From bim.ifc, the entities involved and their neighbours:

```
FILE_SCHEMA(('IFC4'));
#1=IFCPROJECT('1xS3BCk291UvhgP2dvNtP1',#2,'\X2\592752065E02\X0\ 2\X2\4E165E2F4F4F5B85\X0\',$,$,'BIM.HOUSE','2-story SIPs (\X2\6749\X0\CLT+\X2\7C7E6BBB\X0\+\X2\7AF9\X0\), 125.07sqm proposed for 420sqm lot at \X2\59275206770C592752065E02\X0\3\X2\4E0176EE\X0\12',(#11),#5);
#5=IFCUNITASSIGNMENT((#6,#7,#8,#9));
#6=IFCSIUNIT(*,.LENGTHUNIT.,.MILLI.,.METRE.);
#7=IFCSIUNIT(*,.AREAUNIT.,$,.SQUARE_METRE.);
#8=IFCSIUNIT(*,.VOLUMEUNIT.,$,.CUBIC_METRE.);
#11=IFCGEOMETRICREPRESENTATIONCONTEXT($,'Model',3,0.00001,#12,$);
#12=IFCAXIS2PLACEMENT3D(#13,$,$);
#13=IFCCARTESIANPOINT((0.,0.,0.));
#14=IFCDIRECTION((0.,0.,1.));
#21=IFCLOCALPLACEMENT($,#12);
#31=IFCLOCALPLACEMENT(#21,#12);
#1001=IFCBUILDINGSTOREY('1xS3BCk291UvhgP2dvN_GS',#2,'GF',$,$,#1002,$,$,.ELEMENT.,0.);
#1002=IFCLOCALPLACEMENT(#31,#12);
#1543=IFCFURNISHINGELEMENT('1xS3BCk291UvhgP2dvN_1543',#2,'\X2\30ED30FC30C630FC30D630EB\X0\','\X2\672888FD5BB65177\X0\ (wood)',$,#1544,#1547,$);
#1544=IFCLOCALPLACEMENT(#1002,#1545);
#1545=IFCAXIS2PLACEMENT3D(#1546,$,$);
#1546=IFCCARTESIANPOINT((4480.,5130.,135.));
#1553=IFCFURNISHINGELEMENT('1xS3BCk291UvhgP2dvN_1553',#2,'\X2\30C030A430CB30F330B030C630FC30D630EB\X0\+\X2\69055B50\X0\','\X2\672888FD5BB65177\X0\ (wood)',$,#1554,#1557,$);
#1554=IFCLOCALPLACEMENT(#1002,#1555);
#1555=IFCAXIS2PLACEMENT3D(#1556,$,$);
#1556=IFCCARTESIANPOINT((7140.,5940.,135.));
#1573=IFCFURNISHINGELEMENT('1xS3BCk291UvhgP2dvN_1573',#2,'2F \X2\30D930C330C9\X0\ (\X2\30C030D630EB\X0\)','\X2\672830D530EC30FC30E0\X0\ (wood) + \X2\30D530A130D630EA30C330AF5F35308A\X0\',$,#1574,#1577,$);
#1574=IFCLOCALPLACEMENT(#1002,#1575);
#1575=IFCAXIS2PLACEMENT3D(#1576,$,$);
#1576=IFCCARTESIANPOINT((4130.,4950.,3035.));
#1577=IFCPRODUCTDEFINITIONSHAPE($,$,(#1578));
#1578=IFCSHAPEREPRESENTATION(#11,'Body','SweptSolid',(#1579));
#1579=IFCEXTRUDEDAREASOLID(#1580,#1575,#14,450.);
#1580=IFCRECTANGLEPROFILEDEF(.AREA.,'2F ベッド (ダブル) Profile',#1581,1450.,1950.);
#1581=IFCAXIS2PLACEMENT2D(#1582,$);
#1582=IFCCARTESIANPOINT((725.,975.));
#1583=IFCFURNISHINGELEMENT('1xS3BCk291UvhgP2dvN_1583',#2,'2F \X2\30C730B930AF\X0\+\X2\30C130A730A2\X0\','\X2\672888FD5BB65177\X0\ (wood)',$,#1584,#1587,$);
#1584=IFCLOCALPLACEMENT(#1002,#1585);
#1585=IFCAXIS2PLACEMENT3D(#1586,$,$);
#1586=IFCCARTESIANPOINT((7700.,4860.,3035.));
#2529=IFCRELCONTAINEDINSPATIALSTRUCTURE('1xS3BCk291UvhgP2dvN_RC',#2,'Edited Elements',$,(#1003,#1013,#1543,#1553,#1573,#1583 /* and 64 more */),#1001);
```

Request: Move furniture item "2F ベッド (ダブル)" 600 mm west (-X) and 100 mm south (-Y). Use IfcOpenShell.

```python
import ifcopenshell
import ifcopenshell.api.geometry
import ifcopenshell.util.placement
import ifcopenshell.util.unit

model = ifcopenshell.open("bim.ifc")
unit_scale = ifcopenshell.util.unit.calculate_unit_scale(model)

item = model.by_id(1573)
matrix = ifcopenshell.util.placement.get_local_placement(item.ObjectPlacement)
matrix[0, 3] -= 0.6 / unit_scale
matrix[1, 3] -= 0.1 / unit_scale
ifcopenshell.api.geometry.edit_object_placement(model, product=item, matrix=matrix, is_si=False)

print(ifcopenshell.util.placement.get_local_placement(item.ObjectPlacement).round(3) + 0.0)

model.write("bim_edited.ifc")
```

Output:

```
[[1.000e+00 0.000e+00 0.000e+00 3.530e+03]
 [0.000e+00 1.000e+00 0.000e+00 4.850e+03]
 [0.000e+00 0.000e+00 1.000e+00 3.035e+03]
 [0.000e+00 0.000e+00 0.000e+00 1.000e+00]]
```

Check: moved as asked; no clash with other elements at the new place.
